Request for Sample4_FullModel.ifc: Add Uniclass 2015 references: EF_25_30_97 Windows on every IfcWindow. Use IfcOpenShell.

First a look at what the model holds.

```python
import ifcopenshell

model = ifcopenshell.open("Sample4_FullModel.ifc")
print(model.schema)
print("classifications:", [c.Name for c in model.by_type("IfcClassification")])
for ifc_class in ("IfcDoor", "IfcRoof", "IfcStair", "IfcWall", "IfcWindow"):
    print(ifc_class, len(model.by_type(ifc_class)))
```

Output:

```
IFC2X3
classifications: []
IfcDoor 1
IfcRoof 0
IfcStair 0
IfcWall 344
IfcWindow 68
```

```python
import ifcopenshell
import ifcopenshell.api.classification

model = ifcopenshell.open("Sample4_FullModel.ifc")

# IFC2X3 requires Source and Edition and has no link from the project to the system.
system = model.create_entity("IfcClassification", Source="NBS", Edition="2015", Name="Uniclass 2015")

codes = {
    "IfcWindow": ("EF_25_30_97", "Windows"),
}
for ifc_class, (code, name) in codes.items():
    products = model.by_type(ifc_class)
    ifcopenshell.api.classification.add_reference(
        model, products=products, classification=system, identification=code, name=name
    )
    print(code, len(products))

model.write("Sample4_FullModel_edited.ifc")
```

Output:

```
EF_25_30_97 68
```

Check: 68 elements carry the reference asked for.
